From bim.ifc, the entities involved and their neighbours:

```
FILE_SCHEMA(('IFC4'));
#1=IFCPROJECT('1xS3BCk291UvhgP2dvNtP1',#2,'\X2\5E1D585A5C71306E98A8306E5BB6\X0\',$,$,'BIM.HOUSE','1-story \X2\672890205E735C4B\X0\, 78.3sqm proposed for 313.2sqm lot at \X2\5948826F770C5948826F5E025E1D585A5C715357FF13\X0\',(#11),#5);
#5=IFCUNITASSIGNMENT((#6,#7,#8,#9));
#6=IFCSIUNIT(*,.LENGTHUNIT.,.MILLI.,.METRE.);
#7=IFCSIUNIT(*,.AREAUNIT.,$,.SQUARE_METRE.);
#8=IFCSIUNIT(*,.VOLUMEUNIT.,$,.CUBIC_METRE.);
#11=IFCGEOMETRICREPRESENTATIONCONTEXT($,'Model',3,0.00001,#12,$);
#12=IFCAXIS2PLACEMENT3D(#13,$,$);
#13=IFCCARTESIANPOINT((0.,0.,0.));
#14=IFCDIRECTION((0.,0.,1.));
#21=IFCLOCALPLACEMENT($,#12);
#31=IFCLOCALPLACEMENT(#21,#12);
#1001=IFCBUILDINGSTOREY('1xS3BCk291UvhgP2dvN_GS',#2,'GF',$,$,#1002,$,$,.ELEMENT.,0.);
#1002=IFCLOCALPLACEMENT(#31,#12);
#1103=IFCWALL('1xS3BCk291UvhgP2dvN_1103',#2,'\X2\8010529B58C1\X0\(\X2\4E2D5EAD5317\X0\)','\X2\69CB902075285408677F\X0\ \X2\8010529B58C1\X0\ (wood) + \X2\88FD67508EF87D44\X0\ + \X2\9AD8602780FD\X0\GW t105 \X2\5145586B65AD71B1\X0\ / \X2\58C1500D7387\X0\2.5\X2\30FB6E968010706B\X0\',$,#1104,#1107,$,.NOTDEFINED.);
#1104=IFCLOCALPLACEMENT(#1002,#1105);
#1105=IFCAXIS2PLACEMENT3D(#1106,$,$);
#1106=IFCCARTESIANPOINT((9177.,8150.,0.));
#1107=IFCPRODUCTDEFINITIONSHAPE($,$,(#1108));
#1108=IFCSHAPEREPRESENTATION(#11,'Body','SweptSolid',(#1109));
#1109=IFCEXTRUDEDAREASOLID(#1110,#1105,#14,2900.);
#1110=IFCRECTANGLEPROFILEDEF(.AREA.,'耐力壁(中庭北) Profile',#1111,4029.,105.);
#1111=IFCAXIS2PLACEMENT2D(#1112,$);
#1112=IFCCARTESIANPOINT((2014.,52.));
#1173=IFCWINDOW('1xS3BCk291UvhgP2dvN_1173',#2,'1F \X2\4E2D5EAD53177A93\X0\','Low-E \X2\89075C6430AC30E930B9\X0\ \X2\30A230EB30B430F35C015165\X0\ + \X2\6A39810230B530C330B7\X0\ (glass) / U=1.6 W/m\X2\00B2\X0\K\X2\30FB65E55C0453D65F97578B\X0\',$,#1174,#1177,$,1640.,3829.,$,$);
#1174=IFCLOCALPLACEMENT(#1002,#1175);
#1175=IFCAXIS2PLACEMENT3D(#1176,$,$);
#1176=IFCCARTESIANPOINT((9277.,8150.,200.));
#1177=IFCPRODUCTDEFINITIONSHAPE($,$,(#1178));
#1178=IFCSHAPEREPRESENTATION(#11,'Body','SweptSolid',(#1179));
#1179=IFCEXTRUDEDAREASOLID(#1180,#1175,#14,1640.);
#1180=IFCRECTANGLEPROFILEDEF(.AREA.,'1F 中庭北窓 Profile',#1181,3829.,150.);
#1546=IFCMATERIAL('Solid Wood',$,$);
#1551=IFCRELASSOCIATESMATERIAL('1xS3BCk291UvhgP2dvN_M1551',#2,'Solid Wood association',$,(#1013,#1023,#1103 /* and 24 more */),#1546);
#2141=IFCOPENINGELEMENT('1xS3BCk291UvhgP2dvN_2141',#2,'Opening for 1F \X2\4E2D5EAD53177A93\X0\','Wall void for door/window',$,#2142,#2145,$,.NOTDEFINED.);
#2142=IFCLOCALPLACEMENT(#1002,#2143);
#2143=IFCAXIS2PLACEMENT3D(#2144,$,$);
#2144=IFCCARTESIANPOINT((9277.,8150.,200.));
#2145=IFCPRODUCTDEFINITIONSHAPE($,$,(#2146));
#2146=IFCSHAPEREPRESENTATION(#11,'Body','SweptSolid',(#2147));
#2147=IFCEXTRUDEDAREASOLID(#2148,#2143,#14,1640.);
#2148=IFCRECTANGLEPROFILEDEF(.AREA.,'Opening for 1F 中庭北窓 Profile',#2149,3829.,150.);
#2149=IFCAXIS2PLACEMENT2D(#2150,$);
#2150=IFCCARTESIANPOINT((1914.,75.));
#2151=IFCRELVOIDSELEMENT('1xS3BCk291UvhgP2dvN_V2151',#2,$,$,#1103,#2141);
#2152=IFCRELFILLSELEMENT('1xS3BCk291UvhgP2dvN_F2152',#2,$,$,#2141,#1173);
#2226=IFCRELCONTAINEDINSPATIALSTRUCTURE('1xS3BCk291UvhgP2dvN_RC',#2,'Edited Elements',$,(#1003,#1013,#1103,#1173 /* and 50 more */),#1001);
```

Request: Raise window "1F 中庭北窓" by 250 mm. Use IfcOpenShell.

```python
import numpy as np
import ifcopenshell
import ifcopenshell.api.geometry
import ifcopenshell.util.placement
import ifcopenshell.util.unit

model = ifcopenshell.open("bim.ifc")
unit_scale = ifcopenshell.util.unit.calculate_unit_scale(model)

window = model.by_id(1173)
opening = window.FillsVoids[0].RelatingOpeningElement
dz = 250.0

shift = np.array([0.0, 0.0, dz])
# The window is not placed relative to its opening, so move both.
for product in (opening, window):
    matrix = ifcopenshell.util.placement.get_local_placement(product.ObjectPlacement)
    matrix[:3, 3] += shift
    ifcopenshell.api.geometry.edit_object_placement(model, product=product, matrix=matrix, is_si=False)

print(f"moved by {dz * unit_scale:+.3f} m")

model.write("bim_v2.ifc")
```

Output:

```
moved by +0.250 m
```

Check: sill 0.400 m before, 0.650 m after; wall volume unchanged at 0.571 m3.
